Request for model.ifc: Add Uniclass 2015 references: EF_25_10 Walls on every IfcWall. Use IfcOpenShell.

First a look at what the model holds.

```python
import ifcopenshell

model = ifcopenshell.open("model.ifc")
print(model.schema)
print("classifications:", [c.Name for c in model.by_type("IfcClassification")])
for ifc_class in ("IfcDoor", "IfcRoof", "IfcStair", "IfcWall", "IfcWindow"):
    print(ifc_class, len(model.by_type(ifc_class)))
```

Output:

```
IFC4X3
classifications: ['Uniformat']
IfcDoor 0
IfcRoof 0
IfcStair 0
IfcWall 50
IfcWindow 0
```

```python
import ifcopenshell
import ifcopenshell.api.classification

model = ifcopenshell.open("model.ifc")

system = ifcopenshell.api.classification.add_classification(model, classification="Uniclass 2015")

codes = {
    "IfcWall": ("EF_25_10", "Walls"),
}
for ifc_class, (code, name) in codes.items():
    products = model.by_type(ifc_class)
    ifcopenshell.api.classification.add_reference(
        model, products=products, classification=system, identification=code, name=name
    )
    print(code, len(products))

model.write("model_updated.ifc")
```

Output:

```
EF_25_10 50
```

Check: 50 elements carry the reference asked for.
